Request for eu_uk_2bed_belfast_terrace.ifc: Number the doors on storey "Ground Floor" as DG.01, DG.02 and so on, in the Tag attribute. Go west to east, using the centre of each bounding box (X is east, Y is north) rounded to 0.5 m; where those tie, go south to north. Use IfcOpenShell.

First a look at what the model holds.

```python
import ifcopenshell
import ifcopenshell.util.element
import ifcopenshell.util.placement

model = ifcopenshell.open("eu_uk_2bed_belfast_terrace.ifc")
print(model.schema)
storey = next(s for s in model.by_type("IfcBuildingStorey") if s.Name == "Ground Floor")
doors = [e for e in ifcopenshell.util.element.get_decomposition(storey) if e.is_a("IfcDoor")]
for e in sorted(doors, key=lambda e: e.id()):
    origin = ifcopenshell.util.placement.get_local_placement(e.ObjectPlacement)[:3, 3]
    print(e.id(), e.Tag, e.Name, origin.round(2) + 0.0, sep=" | ")
```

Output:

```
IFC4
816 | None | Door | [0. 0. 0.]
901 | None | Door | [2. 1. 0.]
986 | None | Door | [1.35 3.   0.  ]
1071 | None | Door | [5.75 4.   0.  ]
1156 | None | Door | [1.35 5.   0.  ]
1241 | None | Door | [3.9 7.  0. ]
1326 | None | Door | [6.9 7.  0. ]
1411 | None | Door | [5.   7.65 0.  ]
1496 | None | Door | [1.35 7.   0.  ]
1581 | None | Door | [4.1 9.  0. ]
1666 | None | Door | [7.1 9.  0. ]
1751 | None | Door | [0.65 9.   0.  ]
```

```python
import ifcopenshell
import ifcopenshell.geom
import ifcopenshell.util.element
import ifcopenshell.util.shape

model = ifcopenshell.open("eu_uk_2bed_belfast_terrace.ifc")
settings = ifcopenshell.geom.settings()
settings.set("use-world-coords", True)


def centre(element):
    shape = ifcopenshell.geom.create_shape(settings, element)
    return ifcopenshell.util.shape.get_bbox_centroid(shape.geometry)


storey = next(s for s in model.by_type("IfcBuildingStorey") if s.Name == "Ground Floor")
doors = [e for e in ifcopenshell.util.element.get_decomposition(storey) if e.is_a("IfcDoor")]

# Insertion points can sit at a corner or the storey origin, so sort by the geometry (in metres).
centres = {e: centre(e) for e in doors}
doors.sort(key=lambda e: (round(centres[e][0] / 0.5), centres[e][1]))

for i, e in enumerate(doors, start=1):
    number = f"DG.{i:02d}"
    e.Tag = number
    print(e.id(), number)

model.write("eu_uk_2bed_belfast_terrace_v2.ifc")
```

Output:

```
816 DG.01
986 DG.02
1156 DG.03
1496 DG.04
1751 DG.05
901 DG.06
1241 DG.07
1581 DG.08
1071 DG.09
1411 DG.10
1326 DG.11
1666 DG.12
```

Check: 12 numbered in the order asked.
